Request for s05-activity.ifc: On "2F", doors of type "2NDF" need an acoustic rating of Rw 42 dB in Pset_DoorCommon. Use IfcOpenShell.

First a look at what the model holds.

```python
import ifcopenshell
import ifcopenshell.util.element

model = ifcopenshell.open("s05-activity.ifc")
print(model.schema)
storey = next(s for s in model.by_type("IfcBuildingStorey") if s.Name == "2F")
doors = [e for e in ifcopenshell.util.element.get_decomposition(storey) if e.is_a("IfcDoor")]
seen = {}
for e in doors:
    element_type = ifcopenshell.util.element.get_type(e)
    key = (element_type.Name if element_type != e and element_type else None, ifcopenshell.util.element.get_pset(e, "Pset_DoorCommon", "AcousticRating"))
    seen[key] = seen.get(key, 0) + 1
for (name, value), count in sorted(seen.items(), key=str):
    print(count, "x", name, "|", value)
```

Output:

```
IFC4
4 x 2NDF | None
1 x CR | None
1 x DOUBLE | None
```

```python
import ifcopenshell
import ifcopenshell.api.pset
import ifcopenshell.util.element

model = ifcopenshell.open("s05-activity.ifc")

storey = next(s for s in model.by_type("IfcBuildingStorey") if s.Name == "2F")
doors = [e for e in ifcopenshell.util.element.get_decomposition(storey) if e.is_a("IfcDoor")]

count = 0
for e in doors:
    element_type = ifcopenshell.util.element.get_type(e)
    if element_type in (None, e) or element_type.Name != "2NDF":
        continue
    # add_pset returns the element's existing set when there is one.
    pset = ifcopenshell.api.pset.add_pset(model, product=e, name="Pset_DoorCommon")
    ifcopenshell.api.pset.edit_pset(model, pset=pset, properties={"AcousticRating": "Rw 42 dB"})
    count += 1

print(count, "doors updated")

model.write("s05-activity-out.ifc")
```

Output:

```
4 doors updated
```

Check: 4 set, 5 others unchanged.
